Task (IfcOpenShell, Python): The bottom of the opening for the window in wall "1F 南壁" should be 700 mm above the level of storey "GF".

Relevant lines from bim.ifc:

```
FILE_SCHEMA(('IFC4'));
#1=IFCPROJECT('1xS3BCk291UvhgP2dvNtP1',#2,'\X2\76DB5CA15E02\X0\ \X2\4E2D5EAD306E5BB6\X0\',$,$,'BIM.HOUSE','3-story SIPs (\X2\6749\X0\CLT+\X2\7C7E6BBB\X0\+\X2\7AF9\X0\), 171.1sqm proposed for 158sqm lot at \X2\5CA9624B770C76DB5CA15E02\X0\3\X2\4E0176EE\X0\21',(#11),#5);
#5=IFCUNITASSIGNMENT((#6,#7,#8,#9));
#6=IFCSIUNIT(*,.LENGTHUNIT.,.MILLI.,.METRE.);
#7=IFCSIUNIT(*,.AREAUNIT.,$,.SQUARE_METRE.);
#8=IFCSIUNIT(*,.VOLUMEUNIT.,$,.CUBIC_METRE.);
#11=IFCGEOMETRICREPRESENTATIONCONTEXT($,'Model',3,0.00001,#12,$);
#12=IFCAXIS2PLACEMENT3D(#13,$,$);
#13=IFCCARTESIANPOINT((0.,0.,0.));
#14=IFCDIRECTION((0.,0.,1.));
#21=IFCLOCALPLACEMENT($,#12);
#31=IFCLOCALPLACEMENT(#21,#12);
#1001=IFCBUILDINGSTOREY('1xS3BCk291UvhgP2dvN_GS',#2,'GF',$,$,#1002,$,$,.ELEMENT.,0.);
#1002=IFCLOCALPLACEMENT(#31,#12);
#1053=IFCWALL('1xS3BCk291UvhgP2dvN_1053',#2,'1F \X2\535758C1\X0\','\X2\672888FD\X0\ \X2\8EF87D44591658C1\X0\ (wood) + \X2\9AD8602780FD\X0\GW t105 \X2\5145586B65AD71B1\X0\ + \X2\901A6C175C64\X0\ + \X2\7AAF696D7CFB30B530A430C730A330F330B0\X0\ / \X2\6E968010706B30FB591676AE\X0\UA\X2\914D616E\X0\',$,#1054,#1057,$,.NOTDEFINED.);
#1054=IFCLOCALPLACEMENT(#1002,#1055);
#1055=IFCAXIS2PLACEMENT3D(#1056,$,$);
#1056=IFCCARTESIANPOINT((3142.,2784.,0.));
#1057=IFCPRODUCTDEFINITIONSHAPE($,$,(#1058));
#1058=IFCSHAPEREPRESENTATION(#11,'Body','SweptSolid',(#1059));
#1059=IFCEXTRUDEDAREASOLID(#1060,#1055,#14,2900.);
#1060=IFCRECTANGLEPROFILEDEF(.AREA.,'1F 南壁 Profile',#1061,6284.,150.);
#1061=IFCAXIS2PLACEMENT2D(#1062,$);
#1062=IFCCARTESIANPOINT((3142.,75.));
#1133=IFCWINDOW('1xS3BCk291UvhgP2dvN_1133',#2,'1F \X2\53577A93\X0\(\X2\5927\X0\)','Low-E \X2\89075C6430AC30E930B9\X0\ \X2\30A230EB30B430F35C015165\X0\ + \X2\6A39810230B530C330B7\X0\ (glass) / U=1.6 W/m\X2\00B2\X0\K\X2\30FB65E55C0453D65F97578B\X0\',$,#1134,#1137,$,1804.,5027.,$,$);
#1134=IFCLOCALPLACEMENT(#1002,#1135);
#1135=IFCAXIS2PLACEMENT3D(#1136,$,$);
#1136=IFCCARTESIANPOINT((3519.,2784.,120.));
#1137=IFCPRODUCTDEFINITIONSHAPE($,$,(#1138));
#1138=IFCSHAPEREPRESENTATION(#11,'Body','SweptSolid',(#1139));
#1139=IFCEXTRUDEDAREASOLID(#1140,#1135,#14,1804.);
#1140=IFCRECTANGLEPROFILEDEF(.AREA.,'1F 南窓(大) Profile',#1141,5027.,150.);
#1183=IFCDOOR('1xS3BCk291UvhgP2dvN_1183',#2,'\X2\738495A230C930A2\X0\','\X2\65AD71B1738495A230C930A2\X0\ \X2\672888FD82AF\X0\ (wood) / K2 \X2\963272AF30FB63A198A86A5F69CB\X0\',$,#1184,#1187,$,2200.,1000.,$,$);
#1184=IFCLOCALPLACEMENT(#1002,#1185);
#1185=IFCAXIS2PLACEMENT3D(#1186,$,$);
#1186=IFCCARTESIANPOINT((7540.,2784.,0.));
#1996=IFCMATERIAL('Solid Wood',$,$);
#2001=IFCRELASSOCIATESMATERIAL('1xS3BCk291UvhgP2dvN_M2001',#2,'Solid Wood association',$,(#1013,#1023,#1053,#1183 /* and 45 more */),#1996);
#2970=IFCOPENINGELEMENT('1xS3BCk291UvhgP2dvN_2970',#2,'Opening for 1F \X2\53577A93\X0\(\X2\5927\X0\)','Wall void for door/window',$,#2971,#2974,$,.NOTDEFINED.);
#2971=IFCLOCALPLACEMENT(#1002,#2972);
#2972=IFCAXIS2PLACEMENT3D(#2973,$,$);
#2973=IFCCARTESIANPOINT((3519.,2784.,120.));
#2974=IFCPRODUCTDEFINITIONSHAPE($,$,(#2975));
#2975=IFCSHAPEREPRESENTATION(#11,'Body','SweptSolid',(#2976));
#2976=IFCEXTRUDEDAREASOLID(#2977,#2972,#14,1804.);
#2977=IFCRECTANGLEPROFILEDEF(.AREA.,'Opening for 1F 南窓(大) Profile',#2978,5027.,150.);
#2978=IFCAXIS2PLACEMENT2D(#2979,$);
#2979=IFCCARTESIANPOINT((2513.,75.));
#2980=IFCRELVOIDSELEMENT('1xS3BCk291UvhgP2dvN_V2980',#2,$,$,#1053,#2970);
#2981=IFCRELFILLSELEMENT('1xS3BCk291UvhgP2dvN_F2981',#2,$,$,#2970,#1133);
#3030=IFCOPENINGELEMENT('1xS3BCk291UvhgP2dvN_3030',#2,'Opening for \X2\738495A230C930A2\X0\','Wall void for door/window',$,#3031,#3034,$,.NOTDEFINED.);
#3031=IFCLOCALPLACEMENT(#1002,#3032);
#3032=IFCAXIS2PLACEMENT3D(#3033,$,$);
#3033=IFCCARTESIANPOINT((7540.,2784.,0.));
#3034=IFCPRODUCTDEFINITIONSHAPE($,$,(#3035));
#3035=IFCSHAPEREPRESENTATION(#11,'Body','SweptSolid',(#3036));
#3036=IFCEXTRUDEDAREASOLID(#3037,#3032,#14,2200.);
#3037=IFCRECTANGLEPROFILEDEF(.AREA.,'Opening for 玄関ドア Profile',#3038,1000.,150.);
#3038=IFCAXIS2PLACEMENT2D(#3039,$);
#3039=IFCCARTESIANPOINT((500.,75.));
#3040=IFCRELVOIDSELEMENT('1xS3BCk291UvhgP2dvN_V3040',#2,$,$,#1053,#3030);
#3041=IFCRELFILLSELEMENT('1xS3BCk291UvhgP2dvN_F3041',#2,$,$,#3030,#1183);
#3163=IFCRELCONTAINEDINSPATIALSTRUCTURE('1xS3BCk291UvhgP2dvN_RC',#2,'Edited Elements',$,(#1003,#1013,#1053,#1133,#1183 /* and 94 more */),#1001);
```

```python
import numpy as np
import ifcopenshell
import ifcopenshell.api.geometry
import ifcopenshell.geom
import ifcopenshell.util.element
import ifcopenshell.util.placement
import ifcopenshell.util.shape
import ifcopenshell.util.unit

model = ifcopenshell.open("bim.ifc")
unit_scale = ifcopenshell.util.unit.calculate_unit_scale(model)

window = model.by_guid("1xS3BCk291UvhgP2dvN_1133")
opening = window.FillsVoids[0].RelatingOpeningElement
storey = ifcopenshell.util.element.get_container(window, ifc_class="IfcBuildingStorey")
level = ifcopenshell.util.placement.get_local_placement(storey.ObjectPlacement)[2, 3]

# The opening's origin need not be at the sill, so measure its lowest point.
shape = ifcopenshell.geom.create_shape(ifcopenshell.geom.settings(), opening)
bottom = ifcopenshell.util.shape.get_shape_bottom_elevation(shape, shape.geometry) / unit_scale
dz = level + 0.7 / unit_scale - bottom

shift = np.array([0.0, 0.0, dz])
# The window is not placed relative to its opening, so move both.
for product in (opening, window):
    matrix = ifcopenshell.util.placement.get_local_placement(product.ObjectPlacement)
    matrix[:3, 3] += shift
    ifcopenshell.api.geometry.edit_object_placement(model, product=product, matrix=matrix, is_si=False)

print(f"moved by {dz * unit_scale:+.3f} m")

model.write("bim-out.ifc")
```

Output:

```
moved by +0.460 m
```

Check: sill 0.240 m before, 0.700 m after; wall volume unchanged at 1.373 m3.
